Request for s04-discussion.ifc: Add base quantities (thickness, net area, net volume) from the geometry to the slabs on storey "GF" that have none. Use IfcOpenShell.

First a look at what the model holds.

```python
import ifcopenshell
import ifcopenshell.util.element
import ifcopenshell.util.unit

model = ifcopenshell.open("s04-discussion.ifc")
print(model.schema)
for unit_type in ("LENGTHUNIT", "AREAUNIT", "VOLUMEUNIT"):
    print(unit_type, ifcopenshell.util.unit.calculate_unit_scale(model, unit_type))
storey = next(s for s in model.by_type("IfcBuildingStorey") if s.Name == "GF")
slabs = [e for e in ifcopenshell.util.element.get_decomposition(storey) if e.is_a("IfcSlab")]
for e in sorted(slabs, key=lambda e: e.id()):
    print(e.id(), e.is_a(), e.Name, list(ifcopenshell.util.element.get_psets(e, qtos_only=True)), sep=" | ")
```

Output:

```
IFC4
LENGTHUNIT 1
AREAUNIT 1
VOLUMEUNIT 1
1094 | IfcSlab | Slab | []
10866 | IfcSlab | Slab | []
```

```python
import ifcopenshell
import ifcopenshell.api.pset
import ifcopenshell.geom
import ifcopenshell.util.element
import ifcopenshell.util.shape
import ifcopenshell.util.unit

model = ifcopenshell.open("s04-discussion.ifc")
unit_scale = ifcopenshell.util.unit.calculate_unit_scale(model)
area_scale = ifcopenshell.util.unit.calculate_unit_scale(model, "AREAUNIT")
volume_scale = ifcopenshell.util.unit.calculate_unit_scale(model, "VOLUMEUNIT")
settings = ifcopenshell.geom.settings()

storey = next(s for s in model.by_type("IfcBuildingStorey") if s.Name == "GF")
slabs = [e for e in ifcopenshell.util.element.get_decomposition(storey) if e.is_a("IfcSlab")]

for e in sorted(slabs, key=lambda e: e.id()):
    if ifcopenshell.util.element.get_psets(e, qtos_only=True, should_inherit=False):
        continue
    # Geometry comes back in metres, in the element's own axes.
    shape = ifcopenshell.geom.create_shape(settings, e)
    values = {
        "Width": ifcopenshell.util.shape.get_z(shape.geometry) / unit_scale,
        "NetArea": ifcopenshell.util.shape.get_footprint_area(shape.geometry) / area_scale,
        "NetVolume": ifcopenshell.util.shape.get_volume(shape.geometry) / volume_scale,
    }
    qto = ifcopenshell.api.pset.add_qto(model, product=e, name="Qto_SlabBaseQuantities")
    ifcopenshell.api.pset.edit_qto(model, qto=qto, properties=values)
    print(e.id(), {k: round(v, 3) for k, v in values.items()})

model.write("s04-discussion_edited.ifc")
```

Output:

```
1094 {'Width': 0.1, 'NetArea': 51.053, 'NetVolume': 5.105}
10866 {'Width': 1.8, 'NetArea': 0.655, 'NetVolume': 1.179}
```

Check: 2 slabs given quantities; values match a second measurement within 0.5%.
